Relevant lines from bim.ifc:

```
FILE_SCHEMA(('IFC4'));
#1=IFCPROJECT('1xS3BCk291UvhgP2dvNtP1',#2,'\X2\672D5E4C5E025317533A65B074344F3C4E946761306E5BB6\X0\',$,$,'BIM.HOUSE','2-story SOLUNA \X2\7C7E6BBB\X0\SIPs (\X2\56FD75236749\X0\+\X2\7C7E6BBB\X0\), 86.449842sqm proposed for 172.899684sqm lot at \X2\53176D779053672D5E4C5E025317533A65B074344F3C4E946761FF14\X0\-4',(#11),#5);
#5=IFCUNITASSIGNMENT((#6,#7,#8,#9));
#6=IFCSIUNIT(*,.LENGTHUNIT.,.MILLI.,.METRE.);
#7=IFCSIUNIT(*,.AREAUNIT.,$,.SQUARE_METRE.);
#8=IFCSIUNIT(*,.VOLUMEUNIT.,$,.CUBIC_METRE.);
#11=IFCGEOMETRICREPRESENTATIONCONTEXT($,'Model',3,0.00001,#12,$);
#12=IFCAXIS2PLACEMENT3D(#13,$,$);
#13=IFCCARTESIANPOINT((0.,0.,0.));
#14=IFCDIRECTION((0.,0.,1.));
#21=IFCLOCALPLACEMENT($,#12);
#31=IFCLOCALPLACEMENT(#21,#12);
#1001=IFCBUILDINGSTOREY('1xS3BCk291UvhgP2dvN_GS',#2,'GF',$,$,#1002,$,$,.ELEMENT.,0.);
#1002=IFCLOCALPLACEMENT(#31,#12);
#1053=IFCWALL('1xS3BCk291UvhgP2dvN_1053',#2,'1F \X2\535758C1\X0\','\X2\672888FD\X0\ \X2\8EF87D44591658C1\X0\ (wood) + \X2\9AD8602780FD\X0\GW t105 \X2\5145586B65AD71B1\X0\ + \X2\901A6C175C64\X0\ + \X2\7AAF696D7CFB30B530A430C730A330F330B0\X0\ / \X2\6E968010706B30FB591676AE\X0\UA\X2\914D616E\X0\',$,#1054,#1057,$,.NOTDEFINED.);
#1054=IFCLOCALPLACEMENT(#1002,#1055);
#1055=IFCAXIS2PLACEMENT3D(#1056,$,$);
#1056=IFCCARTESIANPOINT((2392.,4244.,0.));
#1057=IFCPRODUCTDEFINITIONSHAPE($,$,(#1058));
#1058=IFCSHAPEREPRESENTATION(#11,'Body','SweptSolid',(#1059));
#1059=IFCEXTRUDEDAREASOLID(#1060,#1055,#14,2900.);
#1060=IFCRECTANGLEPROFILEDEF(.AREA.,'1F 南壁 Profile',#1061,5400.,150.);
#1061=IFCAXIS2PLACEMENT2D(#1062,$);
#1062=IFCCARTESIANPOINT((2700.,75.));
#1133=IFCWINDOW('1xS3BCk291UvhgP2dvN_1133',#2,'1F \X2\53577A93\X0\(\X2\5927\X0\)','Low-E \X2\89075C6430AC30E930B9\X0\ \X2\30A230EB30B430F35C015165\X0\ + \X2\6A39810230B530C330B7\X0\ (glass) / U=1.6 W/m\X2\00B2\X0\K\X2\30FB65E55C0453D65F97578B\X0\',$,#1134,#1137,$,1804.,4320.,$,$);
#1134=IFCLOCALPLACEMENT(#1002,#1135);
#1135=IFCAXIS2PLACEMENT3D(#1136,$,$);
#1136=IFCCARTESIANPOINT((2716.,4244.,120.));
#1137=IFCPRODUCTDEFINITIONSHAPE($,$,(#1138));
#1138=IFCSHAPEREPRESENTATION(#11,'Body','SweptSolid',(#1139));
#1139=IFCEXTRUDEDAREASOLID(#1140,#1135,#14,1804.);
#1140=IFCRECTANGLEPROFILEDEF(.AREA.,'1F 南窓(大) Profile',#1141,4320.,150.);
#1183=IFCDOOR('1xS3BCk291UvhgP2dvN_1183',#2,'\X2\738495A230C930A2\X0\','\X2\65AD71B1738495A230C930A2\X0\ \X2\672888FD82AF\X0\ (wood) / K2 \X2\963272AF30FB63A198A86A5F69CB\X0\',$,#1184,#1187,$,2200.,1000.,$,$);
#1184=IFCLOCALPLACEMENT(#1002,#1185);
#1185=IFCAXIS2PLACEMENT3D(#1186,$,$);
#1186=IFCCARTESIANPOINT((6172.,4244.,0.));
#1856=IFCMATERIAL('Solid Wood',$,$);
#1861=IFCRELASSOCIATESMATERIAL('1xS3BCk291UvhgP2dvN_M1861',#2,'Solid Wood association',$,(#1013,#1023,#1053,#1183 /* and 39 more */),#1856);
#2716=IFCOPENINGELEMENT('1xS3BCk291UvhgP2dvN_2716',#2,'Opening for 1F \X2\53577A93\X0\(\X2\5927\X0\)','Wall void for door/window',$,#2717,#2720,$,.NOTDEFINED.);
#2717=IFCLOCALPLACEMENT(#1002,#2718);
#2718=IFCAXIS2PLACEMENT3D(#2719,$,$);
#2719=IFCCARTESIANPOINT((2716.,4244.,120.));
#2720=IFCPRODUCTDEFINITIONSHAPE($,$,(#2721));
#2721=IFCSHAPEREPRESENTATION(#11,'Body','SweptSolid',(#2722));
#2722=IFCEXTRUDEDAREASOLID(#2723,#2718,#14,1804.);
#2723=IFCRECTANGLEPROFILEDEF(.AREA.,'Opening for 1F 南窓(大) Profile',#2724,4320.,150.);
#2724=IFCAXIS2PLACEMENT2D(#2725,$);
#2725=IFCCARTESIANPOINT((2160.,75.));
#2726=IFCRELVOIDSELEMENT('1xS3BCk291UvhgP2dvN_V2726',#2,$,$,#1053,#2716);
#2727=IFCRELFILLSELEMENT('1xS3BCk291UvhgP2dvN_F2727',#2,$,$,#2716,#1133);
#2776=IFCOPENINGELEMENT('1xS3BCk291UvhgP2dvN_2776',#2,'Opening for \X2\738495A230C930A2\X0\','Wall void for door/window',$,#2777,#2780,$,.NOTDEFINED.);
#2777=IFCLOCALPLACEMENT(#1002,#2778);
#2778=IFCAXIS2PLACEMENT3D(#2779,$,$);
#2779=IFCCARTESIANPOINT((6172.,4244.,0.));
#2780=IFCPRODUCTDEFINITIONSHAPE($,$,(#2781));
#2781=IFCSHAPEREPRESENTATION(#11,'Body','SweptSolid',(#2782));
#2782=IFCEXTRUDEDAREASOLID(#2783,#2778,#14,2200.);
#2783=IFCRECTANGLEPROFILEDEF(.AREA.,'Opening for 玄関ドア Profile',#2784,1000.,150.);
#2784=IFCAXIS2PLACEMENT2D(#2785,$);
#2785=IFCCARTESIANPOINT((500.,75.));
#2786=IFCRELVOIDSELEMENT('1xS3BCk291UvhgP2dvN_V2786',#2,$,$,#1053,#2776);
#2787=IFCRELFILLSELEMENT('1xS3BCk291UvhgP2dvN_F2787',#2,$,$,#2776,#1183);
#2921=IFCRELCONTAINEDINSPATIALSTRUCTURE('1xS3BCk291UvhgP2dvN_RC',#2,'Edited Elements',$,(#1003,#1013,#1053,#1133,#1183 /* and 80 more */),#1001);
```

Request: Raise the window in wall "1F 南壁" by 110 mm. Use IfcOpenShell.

```python
import numpy as np
import ifcopenshell
import ifcopenshell.api.geometry
import ifcopenshell.util.placement
import ifcopenshell.util.unit

model = ifcopenshell.open("bim.ifc")
unit_scale = ifcopenshell.util.unit.calculate_unit_scale(model)

window = model.by_id(1133)
opening = window.FillsVoids[0].RelatingOpeningElement
dz = 0.11 / unit_scale

shift = np.array([0.0, 0.0, dz])
# The window is not placed relative to its opening, so move both.
for product in (opening, window):
    matrix = ifcopenshell.util.placement.get_local_placement(product.ObjectPlacement)
    matrix[:3, 3] += shift
    ifcopenshell.api.geometry.edit_object_placement(model, product=product, matrix=matrix, is_si=False)

print(f"moved by {dz * unit_scale:+.3f} m")

model.write("bim_rev.ifc")
```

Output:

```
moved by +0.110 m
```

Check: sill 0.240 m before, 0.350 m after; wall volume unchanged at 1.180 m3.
